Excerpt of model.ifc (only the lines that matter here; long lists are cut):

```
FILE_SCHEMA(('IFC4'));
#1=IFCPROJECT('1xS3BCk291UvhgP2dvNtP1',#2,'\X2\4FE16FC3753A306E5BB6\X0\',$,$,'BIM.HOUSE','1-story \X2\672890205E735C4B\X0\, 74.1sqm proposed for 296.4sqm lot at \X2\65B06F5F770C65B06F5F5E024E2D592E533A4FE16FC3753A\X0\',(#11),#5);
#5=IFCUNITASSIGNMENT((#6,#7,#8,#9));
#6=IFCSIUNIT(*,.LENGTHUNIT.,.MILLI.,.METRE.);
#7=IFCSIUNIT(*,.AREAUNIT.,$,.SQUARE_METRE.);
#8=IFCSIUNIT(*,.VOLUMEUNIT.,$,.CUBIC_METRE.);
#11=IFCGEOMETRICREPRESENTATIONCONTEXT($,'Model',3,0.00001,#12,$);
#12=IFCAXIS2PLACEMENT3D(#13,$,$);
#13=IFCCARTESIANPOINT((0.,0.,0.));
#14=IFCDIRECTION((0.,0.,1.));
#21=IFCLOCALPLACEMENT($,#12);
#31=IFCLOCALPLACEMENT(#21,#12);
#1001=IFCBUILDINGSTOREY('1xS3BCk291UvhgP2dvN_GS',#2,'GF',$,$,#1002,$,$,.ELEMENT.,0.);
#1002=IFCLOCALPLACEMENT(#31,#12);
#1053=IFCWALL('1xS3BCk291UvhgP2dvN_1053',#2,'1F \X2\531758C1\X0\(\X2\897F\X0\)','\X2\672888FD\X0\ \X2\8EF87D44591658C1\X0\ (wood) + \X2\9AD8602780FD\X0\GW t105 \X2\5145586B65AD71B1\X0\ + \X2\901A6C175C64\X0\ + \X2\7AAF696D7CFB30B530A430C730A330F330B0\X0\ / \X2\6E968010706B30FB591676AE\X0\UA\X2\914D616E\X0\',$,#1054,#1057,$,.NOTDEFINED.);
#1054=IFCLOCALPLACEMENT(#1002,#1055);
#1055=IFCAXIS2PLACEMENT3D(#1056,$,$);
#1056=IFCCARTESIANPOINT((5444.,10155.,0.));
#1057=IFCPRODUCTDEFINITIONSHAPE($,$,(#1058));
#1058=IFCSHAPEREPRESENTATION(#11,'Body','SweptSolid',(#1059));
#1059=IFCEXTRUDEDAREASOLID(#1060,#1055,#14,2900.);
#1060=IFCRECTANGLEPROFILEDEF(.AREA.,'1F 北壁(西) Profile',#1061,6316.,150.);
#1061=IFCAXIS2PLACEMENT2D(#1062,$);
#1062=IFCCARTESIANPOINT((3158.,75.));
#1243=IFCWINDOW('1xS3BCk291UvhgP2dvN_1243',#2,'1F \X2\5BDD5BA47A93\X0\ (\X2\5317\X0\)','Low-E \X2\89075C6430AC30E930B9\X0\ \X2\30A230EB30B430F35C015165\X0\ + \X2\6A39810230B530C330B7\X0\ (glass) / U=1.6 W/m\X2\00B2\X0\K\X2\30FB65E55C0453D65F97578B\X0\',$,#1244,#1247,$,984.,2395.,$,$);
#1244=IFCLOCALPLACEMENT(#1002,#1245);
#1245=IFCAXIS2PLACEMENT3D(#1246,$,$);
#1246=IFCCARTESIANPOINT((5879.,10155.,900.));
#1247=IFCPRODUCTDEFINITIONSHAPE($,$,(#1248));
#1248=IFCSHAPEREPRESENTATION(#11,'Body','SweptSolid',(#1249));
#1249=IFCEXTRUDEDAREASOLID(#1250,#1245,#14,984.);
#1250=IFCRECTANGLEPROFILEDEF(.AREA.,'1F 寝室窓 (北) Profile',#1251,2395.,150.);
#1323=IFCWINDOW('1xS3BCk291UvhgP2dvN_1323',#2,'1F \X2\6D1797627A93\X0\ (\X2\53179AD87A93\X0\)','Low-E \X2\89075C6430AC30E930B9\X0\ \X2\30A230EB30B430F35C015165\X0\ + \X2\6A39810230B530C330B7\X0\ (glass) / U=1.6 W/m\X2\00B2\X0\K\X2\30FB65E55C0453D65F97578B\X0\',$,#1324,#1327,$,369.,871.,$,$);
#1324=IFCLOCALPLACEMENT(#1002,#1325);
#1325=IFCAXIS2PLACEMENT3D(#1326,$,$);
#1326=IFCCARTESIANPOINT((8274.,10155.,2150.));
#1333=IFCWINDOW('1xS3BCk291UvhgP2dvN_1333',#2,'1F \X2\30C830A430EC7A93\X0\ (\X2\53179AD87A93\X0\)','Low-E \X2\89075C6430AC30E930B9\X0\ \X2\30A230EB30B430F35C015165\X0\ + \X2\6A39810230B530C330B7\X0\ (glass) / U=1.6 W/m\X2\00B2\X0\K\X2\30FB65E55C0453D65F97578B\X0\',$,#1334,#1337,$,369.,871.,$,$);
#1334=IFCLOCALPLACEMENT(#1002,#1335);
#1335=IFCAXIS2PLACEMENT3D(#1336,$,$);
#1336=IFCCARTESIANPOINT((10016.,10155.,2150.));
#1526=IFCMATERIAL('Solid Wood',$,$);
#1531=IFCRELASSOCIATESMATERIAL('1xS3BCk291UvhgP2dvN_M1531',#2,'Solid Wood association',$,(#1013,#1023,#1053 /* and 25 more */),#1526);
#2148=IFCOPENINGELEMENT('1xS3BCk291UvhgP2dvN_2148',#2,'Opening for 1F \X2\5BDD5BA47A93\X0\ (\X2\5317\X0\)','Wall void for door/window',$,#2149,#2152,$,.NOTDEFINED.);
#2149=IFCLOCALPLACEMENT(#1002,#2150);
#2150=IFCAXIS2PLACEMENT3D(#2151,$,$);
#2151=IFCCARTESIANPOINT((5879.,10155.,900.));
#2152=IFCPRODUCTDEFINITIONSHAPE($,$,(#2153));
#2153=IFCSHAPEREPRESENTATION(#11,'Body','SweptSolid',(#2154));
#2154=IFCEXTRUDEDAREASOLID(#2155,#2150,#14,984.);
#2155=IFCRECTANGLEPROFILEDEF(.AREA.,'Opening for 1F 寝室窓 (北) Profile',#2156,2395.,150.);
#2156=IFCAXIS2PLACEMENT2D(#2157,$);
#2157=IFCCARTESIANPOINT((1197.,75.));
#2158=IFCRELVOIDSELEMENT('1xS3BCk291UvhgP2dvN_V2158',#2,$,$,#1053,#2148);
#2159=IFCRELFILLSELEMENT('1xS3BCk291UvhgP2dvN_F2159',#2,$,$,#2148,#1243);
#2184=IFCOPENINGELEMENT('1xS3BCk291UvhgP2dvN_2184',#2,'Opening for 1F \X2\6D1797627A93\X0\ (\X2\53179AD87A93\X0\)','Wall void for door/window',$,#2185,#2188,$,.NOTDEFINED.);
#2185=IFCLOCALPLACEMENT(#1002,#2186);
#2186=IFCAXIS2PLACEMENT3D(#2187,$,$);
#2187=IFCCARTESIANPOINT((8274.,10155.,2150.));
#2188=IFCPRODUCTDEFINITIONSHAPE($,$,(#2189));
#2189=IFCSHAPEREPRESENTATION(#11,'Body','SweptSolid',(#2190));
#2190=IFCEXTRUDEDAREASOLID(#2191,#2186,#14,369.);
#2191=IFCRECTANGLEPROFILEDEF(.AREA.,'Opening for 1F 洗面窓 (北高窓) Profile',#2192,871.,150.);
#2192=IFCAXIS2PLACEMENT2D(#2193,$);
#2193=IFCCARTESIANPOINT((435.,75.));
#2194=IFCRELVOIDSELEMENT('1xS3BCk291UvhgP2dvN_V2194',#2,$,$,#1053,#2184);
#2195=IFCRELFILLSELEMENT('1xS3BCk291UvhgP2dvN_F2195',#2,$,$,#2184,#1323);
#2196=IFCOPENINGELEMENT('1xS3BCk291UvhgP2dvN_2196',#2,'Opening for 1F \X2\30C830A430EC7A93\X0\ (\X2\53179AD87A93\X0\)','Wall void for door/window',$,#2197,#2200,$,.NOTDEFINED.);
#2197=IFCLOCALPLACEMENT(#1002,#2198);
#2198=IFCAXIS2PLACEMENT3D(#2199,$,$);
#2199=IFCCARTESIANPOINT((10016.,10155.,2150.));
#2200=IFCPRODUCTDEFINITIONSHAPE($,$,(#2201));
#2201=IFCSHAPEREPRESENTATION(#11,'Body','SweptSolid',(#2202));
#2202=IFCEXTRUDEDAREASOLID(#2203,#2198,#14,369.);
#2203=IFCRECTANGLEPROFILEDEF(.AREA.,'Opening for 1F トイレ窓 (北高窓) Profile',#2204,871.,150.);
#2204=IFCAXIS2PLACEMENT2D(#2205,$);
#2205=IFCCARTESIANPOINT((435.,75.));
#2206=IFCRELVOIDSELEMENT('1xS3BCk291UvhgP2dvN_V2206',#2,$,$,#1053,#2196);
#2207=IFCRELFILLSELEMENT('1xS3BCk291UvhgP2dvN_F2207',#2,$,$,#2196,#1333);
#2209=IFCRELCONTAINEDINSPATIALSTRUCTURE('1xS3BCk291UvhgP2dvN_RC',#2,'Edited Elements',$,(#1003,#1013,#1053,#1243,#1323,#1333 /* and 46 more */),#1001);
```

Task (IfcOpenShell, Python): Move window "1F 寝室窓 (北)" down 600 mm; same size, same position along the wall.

```python
import numpy as np
import ifcopenshell
import ifcopenshell.api.geometry
import ifcopenshell.util.placement
import ifcopenshell.util.unit

model = ifcopenshell.open("model.ifc")
unit_scale = ifcopenshell.util.unit.calculate_unit_scale(model)

window = model.by_guid("1xS3BCk291UvhgP2dvN_1243")
opening = window.FillsVoids[0].RelatingOpeningElement
dz = -0.6 / unit_scale

shift = np.array([0.0, 0.0, dz])
# The window is not placed relative to its opening, so move both.
for product in (opening, window):
    matrix = ifcopenshell.util.placement.get_local_placement(product.ObjectPlacement)
    matrix[:3, 3] += shift
    ifcopenshell.api.geometry.edit_object_placement(model, product=product, matrix=matrix, is_si=False)

print(f"moved by {dz * unit_scale:+.3f} m")

model.write("model_edited.ifc")
```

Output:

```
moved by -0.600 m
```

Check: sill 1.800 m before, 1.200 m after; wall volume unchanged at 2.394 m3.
